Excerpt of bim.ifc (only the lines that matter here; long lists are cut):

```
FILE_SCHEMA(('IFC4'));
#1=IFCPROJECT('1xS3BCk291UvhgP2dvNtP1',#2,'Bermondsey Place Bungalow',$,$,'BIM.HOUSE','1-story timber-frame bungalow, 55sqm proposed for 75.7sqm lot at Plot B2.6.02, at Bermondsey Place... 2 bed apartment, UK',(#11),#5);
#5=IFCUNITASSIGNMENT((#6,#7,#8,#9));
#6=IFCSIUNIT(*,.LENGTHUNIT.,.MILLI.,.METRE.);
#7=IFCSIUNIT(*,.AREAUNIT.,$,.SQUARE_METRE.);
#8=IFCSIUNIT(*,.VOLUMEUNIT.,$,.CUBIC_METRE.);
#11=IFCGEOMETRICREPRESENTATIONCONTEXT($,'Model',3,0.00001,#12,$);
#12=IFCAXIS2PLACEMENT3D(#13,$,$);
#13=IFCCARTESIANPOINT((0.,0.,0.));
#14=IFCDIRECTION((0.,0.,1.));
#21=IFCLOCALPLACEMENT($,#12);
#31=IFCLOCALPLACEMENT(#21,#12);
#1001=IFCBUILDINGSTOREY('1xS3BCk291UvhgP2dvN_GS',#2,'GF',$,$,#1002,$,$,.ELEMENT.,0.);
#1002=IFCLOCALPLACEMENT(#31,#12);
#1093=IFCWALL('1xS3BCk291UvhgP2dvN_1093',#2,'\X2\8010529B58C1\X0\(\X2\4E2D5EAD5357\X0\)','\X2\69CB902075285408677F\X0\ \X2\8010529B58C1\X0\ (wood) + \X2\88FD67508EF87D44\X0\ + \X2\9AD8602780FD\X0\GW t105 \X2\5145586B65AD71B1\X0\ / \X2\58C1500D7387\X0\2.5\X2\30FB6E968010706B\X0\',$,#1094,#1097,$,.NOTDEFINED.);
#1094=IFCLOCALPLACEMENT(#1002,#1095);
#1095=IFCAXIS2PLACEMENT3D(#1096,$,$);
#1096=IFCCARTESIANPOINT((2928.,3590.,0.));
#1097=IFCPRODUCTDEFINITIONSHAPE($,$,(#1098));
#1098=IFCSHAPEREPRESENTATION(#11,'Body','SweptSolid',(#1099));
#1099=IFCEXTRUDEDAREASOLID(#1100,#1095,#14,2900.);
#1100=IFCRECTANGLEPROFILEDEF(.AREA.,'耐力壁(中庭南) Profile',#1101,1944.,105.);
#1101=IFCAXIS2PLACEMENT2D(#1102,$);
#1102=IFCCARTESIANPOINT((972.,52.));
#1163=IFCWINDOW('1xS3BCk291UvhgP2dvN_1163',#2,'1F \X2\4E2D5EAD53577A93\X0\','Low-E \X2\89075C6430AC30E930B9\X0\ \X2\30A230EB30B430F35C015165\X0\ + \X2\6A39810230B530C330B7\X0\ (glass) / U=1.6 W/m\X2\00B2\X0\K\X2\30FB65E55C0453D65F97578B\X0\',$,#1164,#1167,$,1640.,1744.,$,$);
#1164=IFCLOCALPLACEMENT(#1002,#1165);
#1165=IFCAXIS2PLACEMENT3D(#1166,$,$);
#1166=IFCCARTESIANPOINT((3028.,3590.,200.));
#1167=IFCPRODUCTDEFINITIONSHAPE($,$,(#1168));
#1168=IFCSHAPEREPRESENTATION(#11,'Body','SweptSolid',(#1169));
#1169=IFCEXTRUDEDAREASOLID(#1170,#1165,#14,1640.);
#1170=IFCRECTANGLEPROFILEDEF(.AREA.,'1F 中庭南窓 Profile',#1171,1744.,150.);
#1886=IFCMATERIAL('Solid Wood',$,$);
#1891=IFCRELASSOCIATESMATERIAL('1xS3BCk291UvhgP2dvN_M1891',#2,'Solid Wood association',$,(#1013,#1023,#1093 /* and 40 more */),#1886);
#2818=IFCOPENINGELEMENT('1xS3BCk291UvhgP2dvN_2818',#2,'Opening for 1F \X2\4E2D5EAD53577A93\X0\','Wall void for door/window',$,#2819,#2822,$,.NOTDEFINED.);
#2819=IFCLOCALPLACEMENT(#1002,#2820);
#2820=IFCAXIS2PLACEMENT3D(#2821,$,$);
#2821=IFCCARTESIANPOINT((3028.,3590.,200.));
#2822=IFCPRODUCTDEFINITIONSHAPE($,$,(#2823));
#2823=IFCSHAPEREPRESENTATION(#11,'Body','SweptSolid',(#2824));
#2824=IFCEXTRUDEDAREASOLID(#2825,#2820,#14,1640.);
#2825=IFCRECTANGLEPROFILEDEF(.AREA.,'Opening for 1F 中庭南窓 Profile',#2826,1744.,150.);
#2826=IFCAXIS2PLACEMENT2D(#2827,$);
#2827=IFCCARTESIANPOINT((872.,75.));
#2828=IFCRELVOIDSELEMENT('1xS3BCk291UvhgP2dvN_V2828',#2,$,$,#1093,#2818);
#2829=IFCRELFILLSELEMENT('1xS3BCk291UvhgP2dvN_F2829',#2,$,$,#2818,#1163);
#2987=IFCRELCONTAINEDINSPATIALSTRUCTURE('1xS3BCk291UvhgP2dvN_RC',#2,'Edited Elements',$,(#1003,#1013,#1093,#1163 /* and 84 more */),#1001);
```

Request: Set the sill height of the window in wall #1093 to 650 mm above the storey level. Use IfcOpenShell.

```python
import numpy as np
import ifcopenshell
import ifcopenshell.api.geometry
import ifcopenshell.geom
import ifcopenshell.util.element
import ifcopenshell.util.placement
import ifcopenshell.util.shape
import ifcopenshell.util.unit

model = ifcopenshell.open("bim.ifc")
unit_scale = ifcopenshell.util.unit.calculate_unit_scale(model)

window = model.by_guid("1xS3BCk291UvhgP2dvN_1163")
opening = window.FillsVoids[0].RelatingOpeningElement
storey = ifcopenshell.util.element.get_container(window, ifc_class="IfcBuildingStorey")
level = ifcopenshell.util.placement.get_local_placement(storey.ObjectPlacement)[2, 3]

# The opening's origin need not be at the sill, so measure its lowest point.
shape = ifcopenshell.geom.create_shape(ifcopenshell.geom.settings(), opening)
bottom = ifcopenshell.util.shape.get_shape_bottom_elevation(shape, shape.geometry) / unit_scale
dz = level + 0.65 / unit_scale - bottom

shift = np.array([0.0, 0.0, dz])
# The window is not placed relative to its opening, so move both.
for product in (opening, window):
    matrix = ifcopenshell.util.placement.get_local_placement(product.ObjectPlacement)
    matrix[:3, 3] += shift
    ifcopenshell.api.geometry.edit_object_placement(model, product=product, matrix=matrix, is_si=False)

print(f"moved by {dz * unit_scale:+.3f} m")

model.write("bim_updated.ifc")
```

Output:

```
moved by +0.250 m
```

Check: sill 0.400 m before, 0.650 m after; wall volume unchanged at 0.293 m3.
